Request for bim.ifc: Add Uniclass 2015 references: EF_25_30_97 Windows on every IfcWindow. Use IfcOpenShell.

First a look at what the model holds.

```python
import ifcopenshell

model = ifcopenshell.open("bim.ifc")
print(model.schema)
print("classifications:", [c.Name for c in model.by_type("IfcClassification")])
for ifc_class in ("IfcDoor", "IfcRoof", "IfcStair", "IfcWall", "IfcWindow"):
    print(ifc_class, len(model.by_type(ifc_class)))
```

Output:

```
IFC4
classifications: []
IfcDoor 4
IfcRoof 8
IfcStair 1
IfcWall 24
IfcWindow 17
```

```python
import ifcopenshell
import ifcopenshell.api.classification

model = ifcopenshell.open("bim.ifc")

system = ifcopenshell.api.classification.add_classification(model, classification="Uniclass 2015")

codes = {
    "IfcWindow": ("EF_25_30_97", "Windows"),
}
for ifc_class, (code, name) in codes.items():
    products = model.by_type(ifc_class)
    ifcopenshell.api.classification.add_reference(
        model, products=products, classification=system, identification=code, name=name
    )
    print(code, len(products))

model.write("bim_edited.ifc")
```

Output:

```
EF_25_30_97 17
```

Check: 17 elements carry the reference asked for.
